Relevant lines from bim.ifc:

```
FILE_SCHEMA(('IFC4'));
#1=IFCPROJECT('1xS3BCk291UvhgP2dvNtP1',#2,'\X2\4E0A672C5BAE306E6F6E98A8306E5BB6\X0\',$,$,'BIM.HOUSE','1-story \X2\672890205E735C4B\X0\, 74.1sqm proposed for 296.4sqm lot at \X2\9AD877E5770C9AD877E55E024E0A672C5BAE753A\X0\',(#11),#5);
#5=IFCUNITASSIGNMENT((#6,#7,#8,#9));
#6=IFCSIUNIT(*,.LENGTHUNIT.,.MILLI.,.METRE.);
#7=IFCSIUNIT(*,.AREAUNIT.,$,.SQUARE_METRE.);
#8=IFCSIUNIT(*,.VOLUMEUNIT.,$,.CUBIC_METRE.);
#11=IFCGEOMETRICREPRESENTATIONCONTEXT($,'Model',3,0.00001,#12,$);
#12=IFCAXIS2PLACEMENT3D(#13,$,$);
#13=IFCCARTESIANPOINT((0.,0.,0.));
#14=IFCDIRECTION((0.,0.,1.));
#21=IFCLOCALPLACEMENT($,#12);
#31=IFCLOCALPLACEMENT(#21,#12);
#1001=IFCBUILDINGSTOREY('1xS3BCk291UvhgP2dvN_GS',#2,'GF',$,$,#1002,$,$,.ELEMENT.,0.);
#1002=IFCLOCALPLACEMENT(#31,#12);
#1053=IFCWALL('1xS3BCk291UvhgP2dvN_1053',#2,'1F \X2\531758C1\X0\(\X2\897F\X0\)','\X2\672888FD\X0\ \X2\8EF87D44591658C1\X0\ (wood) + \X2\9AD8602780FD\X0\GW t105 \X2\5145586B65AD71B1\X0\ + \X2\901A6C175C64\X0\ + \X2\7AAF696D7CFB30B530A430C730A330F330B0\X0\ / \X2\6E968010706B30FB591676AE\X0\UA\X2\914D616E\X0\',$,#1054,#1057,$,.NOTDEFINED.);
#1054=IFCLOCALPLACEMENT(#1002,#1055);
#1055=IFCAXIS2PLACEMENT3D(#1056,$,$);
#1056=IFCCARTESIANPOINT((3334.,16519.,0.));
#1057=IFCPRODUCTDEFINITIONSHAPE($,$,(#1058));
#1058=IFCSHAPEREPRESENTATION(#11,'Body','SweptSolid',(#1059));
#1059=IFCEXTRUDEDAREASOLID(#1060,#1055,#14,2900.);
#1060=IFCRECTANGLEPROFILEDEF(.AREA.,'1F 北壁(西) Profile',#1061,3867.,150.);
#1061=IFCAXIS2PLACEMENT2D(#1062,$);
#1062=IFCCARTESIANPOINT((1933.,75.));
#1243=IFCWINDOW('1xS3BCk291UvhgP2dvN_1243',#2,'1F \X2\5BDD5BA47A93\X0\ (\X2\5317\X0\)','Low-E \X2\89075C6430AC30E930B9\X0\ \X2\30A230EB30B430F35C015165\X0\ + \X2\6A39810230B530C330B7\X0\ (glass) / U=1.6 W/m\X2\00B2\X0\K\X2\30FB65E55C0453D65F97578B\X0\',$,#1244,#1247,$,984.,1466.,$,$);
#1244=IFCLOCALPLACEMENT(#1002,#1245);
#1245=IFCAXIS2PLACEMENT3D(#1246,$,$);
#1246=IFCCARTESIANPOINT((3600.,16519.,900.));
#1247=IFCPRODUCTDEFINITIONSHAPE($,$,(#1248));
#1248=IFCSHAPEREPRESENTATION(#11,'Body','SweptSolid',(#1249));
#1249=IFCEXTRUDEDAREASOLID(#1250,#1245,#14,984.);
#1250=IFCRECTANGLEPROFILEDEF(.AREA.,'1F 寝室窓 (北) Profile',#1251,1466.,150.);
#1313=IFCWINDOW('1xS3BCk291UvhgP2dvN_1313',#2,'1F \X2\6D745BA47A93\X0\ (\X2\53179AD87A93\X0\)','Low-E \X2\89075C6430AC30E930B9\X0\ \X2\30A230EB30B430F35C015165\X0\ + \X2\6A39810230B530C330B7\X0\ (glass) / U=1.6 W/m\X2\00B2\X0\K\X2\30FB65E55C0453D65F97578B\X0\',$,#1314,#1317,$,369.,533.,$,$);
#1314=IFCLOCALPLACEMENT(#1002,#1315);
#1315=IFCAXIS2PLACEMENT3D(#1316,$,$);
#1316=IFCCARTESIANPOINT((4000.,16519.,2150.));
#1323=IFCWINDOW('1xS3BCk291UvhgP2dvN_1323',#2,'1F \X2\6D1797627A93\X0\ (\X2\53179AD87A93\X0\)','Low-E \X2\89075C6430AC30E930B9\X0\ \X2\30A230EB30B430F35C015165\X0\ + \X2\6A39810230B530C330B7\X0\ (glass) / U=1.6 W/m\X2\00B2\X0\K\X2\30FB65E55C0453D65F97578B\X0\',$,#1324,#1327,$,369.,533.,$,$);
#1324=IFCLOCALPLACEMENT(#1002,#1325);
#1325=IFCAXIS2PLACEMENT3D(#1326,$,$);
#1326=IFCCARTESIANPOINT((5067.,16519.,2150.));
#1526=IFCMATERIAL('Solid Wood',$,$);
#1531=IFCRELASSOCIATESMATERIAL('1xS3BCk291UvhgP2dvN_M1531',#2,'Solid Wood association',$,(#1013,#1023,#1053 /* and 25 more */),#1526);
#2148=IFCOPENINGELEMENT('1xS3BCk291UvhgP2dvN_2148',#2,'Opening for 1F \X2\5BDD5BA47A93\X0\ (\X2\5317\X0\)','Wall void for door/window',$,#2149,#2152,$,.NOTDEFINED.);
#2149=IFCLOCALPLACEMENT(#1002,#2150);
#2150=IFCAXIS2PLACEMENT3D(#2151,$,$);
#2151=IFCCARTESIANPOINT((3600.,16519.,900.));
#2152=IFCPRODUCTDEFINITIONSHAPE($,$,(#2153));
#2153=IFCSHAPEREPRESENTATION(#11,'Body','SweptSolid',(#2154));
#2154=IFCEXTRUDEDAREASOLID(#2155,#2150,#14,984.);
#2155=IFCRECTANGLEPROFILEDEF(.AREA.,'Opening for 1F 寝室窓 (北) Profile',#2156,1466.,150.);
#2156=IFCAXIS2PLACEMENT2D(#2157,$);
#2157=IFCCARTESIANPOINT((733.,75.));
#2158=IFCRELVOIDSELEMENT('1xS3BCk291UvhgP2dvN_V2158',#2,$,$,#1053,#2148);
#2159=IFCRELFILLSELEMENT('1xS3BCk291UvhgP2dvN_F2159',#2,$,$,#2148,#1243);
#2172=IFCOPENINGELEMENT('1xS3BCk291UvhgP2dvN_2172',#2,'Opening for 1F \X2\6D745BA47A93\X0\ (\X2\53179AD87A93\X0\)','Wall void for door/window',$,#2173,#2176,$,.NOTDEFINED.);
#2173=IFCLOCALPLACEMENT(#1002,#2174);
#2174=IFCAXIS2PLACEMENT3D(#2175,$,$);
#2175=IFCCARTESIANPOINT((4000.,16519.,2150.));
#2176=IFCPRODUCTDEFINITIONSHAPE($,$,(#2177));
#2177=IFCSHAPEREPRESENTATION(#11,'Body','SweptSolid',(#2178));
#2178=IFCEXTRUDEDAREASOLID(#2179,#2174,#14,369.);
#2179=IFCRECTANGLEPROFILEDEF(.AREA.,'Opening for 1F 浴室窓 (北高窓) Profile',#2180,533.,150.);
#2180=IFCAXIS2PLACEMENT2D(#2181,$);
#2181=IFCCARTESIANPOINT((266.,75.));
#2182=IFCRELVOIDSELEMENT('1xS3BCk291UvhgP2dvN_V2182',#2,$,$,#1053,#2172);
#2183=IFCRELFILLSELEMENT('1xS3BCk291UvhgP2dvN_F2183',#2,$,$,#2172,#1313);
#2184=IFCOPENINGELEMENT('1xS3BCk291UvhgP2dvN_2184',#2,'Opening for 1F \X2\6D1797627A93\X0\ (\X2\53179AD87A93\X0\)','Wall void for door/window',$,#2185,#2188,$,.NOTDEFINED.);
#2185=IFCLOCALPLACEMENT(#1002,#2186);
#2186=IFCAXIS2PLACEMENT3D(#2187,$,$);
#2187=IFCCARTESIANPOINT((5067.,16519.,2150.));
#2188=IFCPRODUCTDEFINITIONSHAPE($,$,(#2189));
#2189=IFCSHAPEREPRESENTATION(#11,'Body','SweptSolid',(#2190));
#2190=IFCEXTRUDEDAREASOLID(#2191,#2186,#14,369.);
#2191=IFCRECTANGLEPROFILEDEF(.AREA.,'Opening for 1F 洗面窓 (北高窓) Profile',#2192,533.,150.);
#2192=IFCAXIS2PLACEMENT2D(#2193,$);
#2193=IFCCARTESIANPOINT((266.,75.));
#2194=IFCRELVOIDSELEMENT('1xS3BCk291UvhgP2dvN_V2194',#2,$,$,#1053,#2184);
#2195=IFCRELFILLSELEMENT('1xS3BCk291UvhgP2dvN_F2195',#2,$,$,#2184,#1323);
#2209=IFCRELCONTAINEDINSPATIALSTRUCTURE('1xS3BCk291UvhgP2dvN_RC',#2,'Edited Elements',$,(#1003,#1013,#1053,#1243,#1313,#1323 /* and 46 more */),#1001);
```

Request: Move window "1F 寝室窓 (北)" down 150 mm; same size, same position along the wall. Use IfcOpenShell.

```python
import numpy as np
import ifcopenshell
import ifcopenshell.api.geometry
import ifcopenshell.util.placement
import ifcopenshell.util.unit

model = ifcopenshell.open("bim.ifc")
unit_scale = ifcopenshell.util.unit.calculate_unit_scale(model)

window = model.by_id(1243)
opening = window.FillsVoids[0].RelatingOpeningElement
dz = -0.15 / unit_scale

shift = np.array([0.0, 0.0, dz])
# The window is not placed relative to its opening, so move both.
for product in (opening, window):
    matrix = ifcopenshell.util.placement.get_local_placement(product.ObjectPlacement)
    matrix[:3, 3] += shift
    ifcopenshell.api.geometry.edit_object_placement(model, product=product, matrix=matrix, is_si=False)

print(f"moved by {dz * unit_scale:+.3f} m")

model.write("bim_edited.ifc")
```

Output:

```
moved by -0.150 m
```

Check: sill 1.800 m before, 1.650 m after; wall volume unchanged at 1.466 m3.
